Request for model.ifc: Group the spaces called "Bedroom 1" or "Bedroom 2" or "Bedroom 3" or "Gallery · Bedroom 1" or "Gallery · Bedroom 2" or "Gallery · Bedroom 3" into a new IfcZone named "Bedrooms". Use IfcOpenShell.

First a look at what the model holds.

```python
import ifcopenshell

model = ifcopenshell.open("model.ifc")
print(model.schema)
seen = {}
for space in model.by_type("IfcSpace"):
    seen[space.Name] = seen.get(space.Name, 0) + 1
for name, count in sorted(seen.items(), key=str):
    print(count, "x", name)
print("zones:", [z.Name for z in model.by_type("IfcZone")][:20])
```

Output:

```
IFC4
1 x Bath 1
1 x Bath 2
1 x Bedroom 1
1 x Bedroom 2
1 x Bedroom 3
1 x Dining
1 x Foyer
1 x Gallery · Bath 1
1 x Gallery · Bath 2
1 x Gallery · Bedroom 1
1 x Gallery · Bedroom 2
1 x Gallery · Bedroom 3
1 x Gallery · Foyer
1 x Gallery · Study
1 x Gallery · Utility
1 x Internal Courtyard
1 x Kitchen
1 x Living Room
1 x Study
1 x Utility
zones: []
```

```python
import ifcopenshell
import ifcopenshell.api.group
import ifcopenshell.api.root

model = ifcopenshell.open("model.ifc")

names = {"Bedroom 1", "Bedroom 2", "Bedroom 3", "Gallery · Bedroom 1", "Gallery · Bedroom 2", "Gallery · Bedroom 3"}
spaces = [s for s in model.by_type("IfcSpace") if s.Name in names]

zone = ifcopenshell.api.root.create_entity(model, ifc_class="IfcZone", name="Bedrooms")
ifcopenshell.api.group.assign_group(model, products=spaces, group=zone)
print(len(spaces), "spaces in", zone.Name)

model.write("model_updated.ifc")
```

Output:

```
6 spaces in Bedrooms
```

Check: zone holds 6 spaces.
